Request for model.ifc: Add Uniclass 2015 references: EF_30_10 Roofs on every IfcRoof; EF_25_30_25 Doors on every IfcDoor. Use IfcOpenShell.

First a look at what the model holds.

```python
import ifcopenshell

model = ifcopenshell.open("model.ifc")
print(model.schema)
print("classifications:", [c.Name for c in model.by_type("IfcClassification")])
for ifc_class in ("IfcDoor", "IfcRoof", "IfcStair", "IfcWall", "IfcWindow"):
    print(ifc_class, len(model.by_type(ifc_class)))
```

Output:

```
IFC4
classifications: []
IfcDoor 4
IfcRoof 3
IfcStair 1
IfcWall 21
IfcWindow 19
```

```python
import ifcopenshell
import ifcopenshell.api.classification

model = ifcopenshell.open("model.ifc")

system = ifcopenshell.api.classification.add_classification(model, classification="Uniclass 2015")

codes = {
    "IfcRoof": ("EF_30_10", "Roofs"),
    "IfcDoor": ("EF_25_30_25", "Doors"),
}
for ifc_class, (code, name) in codes.items():
    products = model.by_type(ifc_class)
    ifcopenshell.api.classification.add_reference(
        model, products=products, classification=system, identification=code, name=name
    )
    print(code, len(products))

model.write("model_edited.ifc")
```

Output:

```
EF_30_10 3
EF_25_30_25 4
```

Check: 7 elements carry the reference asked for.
